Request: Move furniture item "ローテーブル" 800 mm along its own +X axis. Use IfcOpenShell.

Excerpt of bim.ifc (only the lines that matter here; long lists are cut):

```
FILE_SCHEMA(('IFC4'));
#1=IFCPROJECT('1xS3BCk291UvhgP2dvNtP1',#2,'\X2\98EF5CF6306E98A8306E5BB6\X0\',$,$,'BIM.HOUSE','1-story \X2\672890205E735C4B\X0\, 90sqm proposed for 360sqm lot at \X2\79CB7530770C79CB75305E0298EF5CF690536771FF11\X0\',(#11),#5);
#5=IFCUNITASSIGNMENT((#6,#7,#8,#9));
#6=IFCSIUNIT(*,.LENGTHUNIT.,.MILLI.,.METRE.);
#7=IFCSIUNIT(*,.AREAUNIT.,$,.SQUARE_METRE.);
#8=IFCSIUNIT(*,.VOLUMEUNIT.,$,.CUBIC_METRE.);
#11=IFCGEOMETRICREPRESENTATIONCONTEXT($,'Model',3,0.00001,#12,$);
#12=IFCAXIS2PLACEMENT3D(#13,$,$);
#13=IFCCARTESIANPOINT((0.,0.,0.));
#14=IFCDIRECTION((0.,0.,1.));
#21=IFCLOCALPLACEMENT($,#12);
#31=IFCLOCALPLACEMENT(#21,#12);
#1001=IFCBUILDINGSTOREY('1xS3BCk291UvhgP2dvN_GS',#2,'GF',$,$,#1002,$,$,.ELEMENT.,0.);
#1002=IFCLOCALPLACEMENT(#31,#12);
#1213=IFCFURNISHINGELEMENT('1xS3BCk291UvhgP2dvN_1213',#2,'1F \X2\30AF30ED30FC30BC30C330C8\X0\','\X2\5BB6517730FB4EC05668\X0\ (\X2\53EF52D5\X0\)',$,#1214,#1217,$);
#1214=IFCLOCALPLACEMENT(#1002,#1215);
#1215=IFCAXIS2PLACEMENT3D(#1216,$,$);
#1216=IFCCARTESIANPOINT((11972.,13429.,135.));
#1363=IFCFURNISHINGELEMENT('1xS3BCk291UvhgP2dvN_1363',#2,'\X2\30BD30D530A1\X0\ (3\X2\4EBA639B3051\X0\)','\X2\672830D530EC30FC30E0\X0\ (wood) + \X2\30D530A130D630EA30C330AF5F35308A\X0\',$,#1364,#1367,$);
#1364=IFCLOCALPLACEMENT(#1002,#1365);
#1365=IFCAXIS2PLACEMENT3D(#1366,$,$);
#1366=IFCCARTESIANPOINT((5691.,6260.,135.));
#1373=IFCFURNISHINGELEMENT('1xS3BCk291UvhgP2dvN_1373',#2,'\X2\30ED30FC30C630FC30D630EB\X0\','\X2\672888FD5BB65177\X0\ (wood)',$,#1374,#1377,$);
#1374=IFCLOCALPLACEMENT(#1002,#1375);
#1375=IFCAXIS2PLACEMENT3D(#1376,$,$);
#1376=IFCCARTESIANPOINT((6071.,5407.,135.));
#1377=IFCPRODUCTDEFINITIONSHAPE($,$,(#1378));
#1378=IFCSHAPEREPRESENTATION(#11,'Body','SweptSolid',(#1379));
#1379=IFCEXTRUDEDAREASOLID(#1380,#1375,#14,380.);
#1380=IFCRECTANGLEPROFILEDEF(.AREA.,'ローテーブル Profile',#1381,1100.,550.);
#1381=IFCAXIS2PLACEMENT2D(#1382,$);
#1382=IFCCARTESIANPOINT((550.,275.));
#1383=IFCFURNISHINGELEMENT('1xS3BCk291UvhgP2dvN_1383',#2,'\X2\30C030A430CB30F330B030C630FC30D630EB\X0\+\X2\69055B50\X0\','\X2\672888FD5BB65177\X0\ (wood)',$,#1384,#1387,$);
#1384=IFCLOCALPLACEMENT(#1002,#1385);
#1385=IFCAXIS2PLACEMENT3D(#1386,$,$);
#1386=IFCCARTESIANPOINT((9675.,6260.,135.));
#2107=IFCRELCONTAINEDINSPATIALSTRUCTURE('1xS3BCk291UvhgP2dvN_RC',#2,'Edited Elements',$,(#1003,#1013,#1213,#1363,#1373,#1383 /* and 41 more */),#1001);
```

```python
import ifcopenshell
import ifcopenshell.api.geometry
import ifcopenshell.util.placement

model = ifcopenshell.open("bim.ifc")

item = model.by_guid("1xS3BCk291UvhgP2dvN_1373")
matrix = ifcopenshell.util.placement.get_local_placement(item.ObjectPlacement)
matrix[:3, 3] += matrix[:3, 0] * 800.0
ifcopenshell.api.geometry.edit_object_placement(model, product=item, matrix=matrix, is_si=False)

print(ifcopenshell.util.placement.get_local_placement(item.ObjectPlacement).round(3) + 0.0)

model.write("bim_edited.ifc")
```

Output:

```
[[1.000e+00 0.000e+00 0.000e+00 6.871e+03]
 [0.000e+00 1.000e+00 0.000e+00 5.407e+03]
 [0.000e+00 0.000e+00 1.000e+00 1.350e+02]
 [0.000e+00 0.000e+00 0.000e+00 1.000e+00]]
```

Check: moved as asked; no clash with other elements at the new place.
